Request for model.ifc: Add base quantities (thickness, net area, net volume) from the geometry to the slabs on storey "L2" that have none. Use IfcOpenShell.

First a look at what the model holds.

```python
import ifcopenshell
import ifcopenshell.util.element
import ifcopenshell.util.unit

model = ifcopenshell.open("model.ifc")
print(model.schema)
for unit_type in ("LENGTHUNIT", "AREAUNIT", "VOLUMEUNIT"):
    print(unit_type, ifcopenshell.util.unit.calculate_unit_scale(model, unit_type))
storey = next(s for s in model.by_type("IfcBuildingStorey") if s.Name == "L2")
slabs = [e for e in ifcopenshell.util.element.get_decomposition(storey) if e.is_a("IfcSlab")]
for e in sorted(slabs, key=lambda e: e.id()):
    print(e.id(), e.is_a(), e.Name, list(ifcopenshell.util.element.get_psets(e, qtos_only=True)), sep=" | ")
```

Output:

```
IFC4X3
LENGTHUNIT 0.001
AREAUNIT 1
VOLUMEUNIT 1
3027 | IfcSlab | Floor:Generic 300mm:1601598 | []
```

```python
import ifcopenshell
import ifcopenshell.api.pset
import ifcopenshell.geom
import ifcopenshell.util.element
import ifcopenshell.util.shape
import ifcopenshell.util.unit

model = ifcopenshell.open("model.ifc")
unit_scale = ifcopenshell.util.unit.calculate_unit_scale(model)
area_scale = ifcopenshell.util.unit.calculate_unit_scale(model, "AREAUNIT")
volume_scale = ifcopenshell.util.unit.calculate_unit_scale(model, "VOLUMEUNIT")
settings = ifcopenshell.geom.settings()

storey = next(s for s in model.by_type("IfcBuildingStorey") if s.Name == "L2")
slabs = [e for e in ifcopenshell.util.element.get_decomposition(storey) if e.is_a("IfcSlab")]

for e in sorted(slabs, key=lambda e: e.id()):
    if ifcopenshell.util.element.get_psets(e, qtos_only=True, should_inherit=False):
        continue
    # Geometry comes back in metres, in the element's own axes.
    shape = ifcopenshell.geom.create_shape(settings, e)
    values = {
        "Width": ifcopenshell.util.shape.get_z(shape.geometry) / unit_scale,
        "NetArea": ifcopenshell.util.shape.get_footprint_area(shape.geometry) / area_scale,
        "NetVolume": ifcopenshell.util.shape.get_volume(shape.geometry) / volume_scale,
    }
    qto = ifcopenshell.api.pset.add_qto(model, product=e, name="Qto_SlabBaseQuantities")
    ifcopenshell.api.pset.edit_qto(model, qto=qto, properties=values)
    print(e.id(), {k: round(v, 3) for k, v in values.items()})

model.write("model_rev.ifc")
```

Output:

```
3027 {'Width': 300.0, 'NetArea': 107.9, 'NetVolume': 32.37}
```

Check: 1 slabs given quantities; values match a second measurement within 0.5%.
